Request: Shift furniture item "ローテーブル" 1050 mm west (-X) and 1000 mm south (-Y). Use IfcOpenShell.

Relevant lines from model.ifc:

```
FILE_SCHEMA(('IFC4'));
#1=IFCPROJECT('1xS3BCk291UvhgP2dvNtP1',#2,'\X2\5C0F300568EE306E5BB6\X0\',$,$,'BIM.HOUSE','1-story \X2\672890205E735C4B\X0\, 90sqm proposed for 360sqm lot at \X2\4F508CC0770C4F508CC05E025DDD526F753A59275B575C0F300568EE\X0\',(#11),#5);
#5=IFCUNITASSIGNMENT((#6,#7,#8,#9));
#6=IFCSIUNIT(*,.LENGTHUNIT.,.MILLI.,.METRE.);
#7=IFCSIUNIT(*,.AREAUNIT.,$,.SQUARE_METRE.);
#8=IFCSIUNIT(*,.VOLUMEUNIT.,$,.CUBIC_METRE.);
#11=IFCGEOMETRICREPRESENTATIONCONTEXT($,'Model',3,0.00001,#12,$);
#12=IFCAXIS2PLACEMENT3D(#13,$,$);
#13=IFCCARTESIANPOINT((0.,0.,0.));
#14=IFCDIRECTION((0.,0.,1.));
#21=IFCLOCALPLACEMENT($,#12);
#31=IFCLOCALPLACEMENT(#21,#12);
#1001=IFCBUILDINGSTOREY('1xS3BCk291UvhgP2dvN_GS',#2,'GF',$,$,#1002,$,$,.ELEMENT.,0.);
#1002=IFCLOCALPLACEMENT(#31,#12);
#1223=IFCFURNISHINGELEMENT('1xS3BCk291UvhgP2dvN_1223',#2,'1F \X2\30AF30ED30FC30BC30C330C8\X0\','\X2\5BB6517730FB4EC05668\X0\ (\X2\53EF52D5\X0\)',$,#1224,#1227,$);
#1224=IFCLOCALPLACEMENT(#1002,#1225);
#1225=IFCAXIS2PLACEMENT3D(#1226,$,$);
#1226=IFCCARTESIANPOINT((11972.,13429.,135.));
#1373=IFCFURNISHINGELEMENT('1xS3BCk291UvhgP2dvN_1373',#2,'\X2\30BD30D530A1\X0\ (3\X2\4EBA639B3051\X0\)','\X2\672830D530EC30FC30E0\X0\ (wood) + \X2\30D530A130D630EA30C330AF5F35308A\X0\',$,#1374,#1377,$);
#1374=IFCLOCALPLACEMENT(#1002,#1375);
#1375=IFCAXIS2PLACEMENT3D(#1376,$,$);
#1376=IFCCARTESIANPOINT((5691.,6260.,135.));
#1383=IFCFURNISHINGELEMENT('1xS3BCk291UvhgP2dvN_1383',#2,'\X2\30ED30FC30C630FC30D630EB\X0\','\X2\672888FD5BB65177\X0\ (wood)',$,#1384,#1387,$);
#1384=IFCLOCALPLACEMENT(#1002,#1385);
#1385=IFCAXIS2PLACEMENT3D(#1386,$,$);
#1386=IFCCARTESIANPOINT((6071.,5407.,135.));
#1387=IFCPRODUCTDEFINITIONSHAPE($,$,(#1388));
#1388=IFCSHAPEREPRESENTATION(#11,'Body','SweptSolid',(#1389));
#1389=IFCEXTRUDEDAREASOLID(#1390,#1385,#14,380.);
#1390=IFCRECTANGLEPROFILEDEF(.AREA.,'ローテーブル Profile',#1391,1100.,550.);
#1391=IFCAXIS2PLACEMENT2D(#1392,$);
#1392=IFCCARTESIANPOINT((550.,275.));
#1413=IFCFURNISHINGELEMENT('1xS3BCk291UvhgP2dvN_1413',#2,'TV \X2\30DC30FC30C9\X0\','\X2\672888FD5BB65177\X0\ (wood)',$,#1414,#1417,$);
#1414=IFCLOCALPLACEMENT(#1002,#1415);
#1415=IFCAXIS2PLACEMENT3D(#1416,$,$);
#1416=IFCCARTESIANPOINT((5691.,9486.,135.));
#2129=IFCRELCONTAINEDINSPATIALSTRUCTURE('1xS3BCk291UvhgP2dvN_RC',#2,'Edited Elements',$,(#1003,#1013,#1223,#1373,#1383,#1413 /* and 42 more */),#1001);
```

```python
import ifcopenshell
import ifcopenshell.api.geometry
import ifcopenshell.util.placement
import ifcopenshell.util.unit

model = ifcopenshell.open("model.ifc")
unit_scale = ifcopenshell.util.unit.calculate_unit_scale(model)

item = model.by_guid("1xS3BCk291UvhgP2dvN_1383")
matrix = ifcopenshell.util.placement.get_local_placement(item.ObjectPlacement)
matrix[0, 3] -= 1.05 / unit_scale
matrix[1, 3] -= 1 / unit_scale
ifcopenshell.api.geometry.edit_object_placement(model, product=item, matrix=matrix, is_si=False)

print(ifcopenshell.util.placement.get_local_placement(item.ObjectPlacement).round(3) + 0.0)

model.write("model_updated.ifc")
```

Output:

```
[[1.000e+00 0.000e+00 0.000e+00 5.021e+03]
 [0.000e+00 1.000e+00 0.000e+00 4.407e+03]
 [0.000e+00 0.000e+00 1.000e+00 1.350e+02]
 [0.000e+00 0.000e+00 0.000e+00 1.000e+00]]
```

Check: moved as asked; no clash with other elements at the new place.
